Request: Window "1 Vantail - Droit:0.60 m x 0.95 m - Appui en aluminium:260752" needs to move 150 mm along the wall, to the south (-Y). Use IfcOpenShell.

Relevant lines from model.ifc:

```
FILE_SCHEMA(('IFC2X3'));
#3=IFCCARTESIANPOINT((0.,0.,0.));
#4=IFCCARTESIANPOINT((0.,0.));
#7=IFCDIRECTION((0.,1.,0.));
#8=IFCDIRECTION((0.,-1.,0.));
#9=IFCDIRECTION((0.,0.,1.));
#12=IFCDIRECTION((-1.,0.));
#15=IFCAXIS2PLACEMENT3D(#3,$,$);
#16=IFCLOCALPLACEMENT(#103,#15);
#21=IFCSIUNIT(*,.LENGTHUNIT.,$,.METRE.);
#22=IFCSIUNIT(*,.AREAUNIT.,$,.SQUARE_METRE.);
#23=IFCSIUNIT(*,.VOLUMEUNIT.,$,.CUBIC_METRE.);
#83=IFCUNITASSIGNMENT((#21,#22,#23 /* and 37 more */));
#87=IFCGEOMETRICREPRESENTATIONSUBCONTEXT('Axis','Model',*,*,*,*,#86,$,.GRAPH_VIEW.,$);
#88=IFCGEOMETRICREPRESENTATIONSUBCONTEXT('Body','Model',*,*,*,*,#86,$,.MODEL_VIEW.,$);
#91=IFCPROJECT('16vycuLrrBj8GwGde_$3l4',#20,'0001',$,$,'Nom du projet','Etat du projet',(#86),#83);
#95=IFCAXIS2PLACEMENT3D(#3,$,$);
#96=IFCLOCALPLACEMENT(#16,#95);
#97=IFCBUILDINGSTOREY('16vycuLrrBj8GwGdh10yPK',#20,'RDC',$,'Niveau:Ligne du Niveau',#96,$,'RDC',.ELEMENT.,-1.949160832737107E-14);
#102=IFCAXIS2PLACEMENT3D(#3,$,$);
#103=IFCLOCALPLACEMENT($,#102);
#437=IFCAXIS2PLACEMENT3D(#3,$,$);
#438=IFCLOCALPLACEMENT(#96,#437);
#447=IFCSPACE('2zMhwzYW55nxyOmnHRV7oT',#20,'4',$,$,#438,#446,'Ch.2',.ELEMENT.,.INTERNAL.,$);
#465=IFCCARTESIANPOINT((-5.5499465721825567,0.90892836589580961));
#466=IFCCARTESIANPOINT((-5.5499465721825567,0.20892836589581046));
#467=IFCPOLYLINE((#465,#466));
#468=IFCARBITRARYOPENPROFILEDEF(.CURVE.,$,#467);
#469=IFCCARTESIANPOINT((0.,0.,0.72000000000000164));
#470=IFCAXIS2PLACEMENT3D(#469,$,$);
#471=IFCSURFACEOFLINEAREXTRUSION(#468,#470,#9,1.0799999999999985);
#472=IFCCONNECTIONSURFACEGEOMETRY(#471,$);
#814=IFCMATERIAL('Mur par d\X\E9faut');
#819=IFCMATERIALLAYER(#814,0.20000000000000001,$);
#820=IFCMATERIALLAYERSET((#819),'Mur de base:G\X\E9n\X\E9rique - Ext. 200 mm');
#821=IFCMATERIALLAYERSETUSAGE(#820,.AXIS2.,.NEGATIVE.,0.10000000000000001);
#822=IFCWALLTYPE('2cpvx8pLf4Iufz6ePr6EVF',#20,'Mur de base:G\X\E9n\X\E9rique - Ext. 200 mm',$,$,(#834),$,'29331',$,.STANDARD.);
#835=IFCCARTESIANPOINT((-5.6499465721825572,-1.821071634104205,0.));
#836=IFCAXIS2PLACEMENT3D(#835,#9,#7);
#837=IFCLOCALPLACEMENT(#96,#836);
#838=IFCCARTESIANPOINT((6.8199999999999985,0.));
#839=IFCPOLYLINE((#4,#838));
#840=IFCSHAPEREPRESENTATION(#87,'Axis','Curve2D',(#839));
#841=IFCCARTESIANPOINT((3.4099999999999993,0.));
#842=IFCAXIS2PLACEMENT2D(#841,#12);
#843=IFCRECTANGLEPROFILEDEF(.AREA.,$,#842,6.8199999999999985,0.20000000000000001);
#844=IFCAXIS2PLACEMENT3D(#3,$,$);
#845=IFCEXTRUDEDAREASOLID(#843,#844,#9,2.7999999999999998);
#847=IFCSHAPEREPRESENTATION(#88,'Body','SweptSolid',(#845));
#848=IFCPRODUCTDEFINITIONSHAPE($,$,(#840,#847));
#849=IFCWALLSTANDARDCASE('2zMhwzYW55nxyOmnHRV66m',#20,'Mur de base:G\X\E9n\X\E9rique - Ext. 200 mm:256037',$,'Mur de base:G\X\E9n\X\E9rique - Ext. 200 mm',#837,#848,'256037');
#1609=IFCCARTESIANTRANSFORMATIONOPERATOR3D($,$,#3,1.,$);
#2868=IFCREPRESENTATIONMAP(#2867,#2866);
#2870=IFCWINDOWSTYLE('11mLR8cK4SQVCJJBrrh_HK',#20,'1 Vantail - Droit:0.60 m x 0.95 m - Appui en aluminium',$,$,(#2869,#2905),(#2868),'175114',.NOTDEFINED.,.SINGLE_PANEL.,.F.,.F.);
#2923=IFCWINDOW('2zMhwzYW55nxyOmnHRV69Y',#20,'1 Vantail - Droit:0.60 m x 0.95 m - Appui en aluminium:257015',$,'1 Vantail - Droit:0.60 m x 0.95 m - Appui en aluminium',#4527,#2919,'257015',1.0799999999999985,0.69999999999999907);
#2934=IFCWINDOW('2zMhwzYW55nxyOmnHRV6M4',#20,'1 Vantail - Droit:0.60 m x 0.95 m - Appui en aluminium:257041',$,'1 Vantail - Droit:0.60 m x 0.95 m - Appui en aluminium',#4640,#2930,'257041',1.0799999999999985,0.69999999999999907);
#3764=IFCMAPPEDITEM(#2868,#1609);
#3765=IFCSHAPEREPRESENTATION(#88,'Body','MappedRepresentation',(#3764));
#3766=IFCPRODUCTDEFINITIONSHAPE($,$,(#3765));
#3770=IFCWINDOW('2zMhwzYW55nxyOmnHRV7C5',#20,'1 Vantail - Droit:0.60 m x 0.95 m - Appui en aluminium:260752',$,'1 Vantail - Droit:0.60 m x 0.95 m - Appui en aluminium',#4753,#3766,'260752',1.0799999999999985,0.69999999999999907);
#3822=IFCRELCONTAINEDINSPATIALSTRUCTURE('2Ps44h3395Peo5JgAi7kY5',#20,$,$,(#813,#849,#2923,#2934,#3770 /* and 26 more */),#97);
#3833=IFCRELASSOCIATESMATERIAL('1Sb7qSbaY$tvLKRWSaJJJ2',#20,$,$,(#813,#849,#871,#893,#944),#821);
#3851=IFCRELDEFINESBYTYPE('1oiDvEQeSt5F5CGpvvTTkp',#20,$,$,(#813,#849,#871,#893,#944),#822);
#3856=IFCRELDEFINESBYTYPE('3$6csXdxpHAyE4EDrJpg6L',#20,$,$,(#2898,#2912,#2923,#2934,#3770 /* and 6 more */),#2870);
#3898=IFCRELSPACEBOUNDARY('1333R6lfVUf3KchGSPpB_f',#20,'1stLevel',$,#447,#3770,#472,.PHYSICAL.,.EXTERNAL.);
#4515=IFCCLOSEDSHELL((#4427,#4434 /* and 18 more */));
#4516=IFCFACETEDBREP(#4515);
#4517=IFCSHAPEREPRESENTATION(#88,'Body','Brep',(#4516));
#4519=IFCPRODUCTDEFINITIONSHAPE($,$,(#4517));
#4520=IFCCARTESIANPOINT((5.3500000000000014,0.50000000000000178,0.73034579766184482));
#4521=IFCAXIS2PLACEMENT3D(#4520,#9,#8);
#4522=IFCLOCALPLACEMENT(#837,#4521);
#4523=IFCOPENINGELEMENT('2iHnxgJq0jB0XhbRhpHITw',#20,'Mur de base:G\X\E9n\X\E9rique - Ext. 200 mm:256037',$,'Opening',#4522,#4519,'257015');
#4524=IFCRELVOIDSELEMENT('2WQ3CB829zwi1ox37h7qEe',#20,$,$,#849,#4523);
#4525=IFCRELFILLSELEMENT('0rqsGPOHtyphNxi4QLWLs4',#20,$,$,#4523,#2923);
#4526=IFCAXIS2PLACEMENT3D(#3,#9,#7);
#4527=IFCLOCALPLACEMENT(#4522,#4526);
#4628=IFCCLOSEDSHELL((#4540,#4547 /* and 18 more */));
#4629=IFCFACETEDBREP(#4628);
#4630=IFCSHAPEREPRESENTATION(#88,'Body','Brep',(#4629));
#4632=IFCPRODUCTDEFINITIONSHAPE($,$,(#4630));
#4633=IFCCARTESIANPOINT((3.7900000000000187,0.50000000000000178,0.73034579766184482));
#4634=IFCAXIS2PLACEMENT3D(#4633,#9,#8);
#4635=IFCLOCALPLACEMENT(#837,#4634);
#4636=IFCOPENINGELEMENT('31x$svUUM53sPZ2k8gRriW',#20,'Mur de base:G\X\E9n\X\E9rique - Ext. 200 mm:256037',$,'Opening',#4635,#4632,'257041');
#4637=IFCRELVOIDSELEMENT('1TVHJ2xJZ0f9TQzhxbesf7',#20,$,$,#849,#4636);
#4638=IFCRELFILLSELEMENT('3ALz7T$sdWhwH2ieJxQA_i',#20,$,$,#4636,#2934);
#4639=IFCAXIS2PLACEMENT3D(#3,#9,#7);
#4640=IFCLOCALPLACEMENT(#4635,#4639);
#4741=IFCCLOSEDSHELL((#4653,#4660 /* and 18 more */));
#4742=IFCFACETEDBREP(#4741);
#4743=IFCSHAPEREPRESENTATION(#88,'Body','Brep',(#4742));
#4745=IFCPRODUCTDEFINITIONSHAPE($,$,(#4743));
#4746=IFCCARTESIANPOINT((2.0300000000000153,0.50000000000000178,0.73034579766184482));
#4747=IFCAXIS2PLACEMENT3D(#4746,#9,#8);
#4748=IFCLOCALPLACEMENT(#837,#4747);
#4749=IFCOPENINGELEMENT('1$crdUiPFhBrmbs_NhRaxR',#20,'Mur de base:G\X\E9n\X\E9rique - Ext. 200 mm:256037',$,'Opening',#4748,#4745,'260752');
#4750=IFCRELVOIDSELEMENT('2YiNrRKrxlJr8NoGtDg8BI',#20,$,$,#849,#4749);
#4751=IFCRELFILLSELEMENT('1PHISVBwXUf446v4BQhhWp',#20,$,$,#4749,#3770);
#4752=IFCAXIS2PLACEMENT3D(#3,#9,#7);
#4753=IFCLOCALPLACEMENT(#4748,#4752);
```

```python
import numpy as np
import ifcopenshell
import ifcopenshell.api.geometry
import ifcopenshell.util.placement

model = ifcopenshell.open("model.ifc")

window = model.by_id(3770)
opening = window.FillsVoids[0].RelatingOpeningElement
wall = opening.VoidsElements[0].RelatingBuildingElement

wall_matrix = ifcopenshell.util.placement.get_local_placement(wall.ObjectPlacement)
shift = wall_matrix[:3, 0] * -0.15
before = ifcopenshell.util.placement.get_local_placement(window.ObjectPlacement)[:3, 3].copy()

# The window is placed relative to its opening, so it follows when the opening moves.
matrix = ifcopenshell.util.placement.get_local_placement(opening.ObjectPlacement)
matrix[:3, 3] += shift
ifcopenshell.api.geometry.edit_object_placement(
    model, product=opening, matrix=matrix, is_si=False, should_transform_children=True
)

# Space boundary surfaces are stored in each space's coordinates; move them too.
for rel in window.ProvidesBoundaries:
    if not rel.ConnectionGeometry:
        continue
    surface = rel.ConnectionGeometry.SurfaceOnRelatingElement
    space_matrix = ifcopenshell.util.placement.get_local_placement(rel.RelatingSpace.ObjectPlacement)
    point = np.array(surface.Position.Location.Coordinates) + space_matrix[:3, :3].T @ shift
    surface.Position = model.createIfcAxis2Placement3D(
        model.createIfcCartesianPoint(point.tolist()), surface.Position.Axis, surface.Position.RefDirection
    )

after = ifcopenshell.util.placement.get_local_placement(window.ObjectPlacement)[:3, 3]
print("window moved by", (after - before).round(3) + 0.0)

model.write("model-out.ifc")
```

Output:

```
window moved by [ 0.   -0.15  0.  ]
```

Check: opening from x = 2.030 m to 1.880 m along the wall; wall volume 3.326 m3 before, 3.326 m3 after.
